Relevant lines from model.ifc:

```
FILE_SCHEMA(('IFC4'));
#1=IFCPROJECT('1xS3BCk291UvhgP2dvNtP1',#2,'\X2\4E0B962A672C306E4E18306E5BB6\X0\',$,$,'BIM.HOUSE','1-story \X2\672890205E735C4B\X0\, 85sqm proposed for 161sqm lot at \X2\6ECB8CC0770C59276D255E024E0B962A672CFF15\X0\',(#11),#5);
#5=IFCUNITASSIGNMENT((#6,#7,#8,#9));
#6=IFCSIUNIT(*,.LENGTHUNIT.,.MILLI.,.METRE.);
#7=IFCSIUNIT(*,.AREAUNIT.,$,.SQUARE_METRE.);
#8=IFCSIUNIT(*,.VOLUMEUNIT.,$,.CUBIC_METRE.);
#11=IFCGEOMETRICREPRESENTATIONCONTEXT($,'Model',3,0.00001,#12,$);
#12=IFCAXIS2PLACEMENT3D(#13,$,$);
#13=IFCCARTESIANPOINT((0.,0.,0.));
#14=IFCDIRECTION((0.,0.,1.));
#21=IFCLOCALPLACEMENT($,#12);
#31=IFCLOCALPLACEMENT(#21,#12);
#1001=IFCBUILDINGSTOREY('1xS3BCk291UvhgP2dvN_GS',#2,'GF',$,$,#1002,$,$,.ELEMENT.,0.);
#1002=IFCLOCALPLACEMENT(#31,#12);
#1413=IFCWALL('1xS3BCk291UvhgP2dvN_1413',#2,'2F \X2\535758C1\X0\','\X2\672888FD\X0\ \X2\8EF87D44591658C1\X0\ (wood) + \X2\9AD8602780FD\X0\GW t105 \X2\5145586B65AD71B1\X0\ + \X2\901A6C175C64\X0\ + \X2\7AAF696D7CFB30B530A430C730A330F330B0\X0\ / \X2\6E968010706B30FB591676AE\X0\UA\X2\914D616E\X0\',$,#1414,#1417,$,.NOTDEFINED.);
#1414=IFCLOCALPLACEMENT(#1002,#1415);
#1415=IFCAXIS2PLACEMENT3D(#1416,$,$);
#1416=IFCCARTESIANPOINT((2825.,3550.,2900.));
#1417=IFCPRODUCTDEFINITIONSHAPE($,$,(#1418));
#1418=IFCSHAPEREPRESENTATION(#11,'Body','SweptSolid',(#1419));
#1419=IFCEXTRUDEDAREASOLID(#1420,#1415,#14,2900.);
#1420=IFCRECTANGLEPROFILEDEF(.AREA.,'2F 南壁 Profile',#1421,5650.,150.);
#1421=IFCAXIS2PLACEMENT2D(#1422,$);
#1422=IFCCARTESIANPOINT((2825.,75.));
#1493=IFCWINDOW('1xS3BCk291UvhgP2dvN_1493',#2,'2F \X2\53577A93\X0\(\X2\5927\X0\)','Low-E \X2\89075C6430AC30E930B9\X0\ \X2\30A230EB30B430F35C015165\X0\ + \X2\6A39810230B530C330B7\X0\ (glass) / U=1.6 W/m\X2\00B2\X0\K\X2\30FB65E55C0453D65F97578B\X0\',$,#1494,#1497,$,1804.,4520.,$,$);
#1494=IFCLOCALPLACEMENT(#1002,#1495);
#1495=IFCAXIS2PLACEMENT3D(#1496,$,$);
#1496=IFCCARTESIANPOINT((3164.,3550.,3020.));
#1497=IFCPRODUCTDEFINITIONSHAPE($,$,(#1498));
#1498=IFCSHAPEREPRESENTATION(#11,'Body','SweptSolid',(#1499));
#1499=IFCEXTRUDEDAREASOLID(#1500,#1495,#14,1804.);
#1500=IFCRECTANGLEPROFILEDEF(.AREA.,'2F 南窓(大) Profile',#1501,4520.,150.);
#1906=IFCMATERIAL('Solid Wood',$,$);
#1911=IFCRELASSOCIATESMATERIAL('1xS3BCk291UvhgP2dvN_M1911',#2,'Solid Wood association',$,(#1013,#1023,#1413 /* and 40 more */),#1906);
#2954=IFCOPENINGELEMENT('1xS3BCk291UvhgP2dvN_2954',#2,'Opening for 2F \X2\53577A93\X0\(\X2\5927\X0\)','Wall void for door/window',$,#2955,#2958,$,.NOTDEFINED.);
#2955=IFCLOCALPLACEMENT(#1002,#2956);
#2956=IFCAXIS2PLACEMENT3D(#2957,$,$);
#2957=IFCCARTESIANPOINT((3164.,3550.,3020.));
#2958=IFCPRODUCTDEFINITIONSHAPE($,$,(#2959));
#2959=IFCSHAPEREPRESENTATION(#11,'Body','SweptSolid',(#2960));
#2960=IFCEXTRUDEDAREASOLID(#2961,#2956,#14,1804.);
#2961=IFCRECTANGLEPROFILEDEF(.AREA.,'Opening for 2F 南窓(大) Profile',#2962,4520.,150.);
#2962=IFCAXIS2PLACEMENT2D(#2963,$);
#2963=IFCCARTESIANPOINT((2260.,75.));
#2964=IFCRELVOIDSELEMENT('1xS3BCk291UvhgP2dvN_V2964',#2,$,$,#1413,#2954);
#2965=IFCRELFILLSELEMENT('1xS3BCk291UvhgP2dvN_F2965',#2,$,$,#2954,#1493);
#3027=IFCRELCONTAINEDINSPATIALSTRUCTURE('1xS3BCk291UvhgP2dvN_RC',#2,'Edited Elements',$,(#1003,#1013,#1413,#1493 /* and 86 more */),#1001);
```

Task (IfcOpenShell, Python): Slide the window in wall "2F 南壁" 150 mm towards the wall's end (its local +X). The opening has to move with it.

```python
import ifcopenshell
import ifcopenshell.api.geometry
import ifcopenshell.util.placement

model = ifcopenshell.open("model.ifc")

window = model.by_id(1493)
opening = window.FillsVoids[0].RelatingOpeningElement
wall = opening.VoidsElements[0].RelatingBuildingElement

wall_matrix = ifcopenshell.util.placement.get_local_placement(wall.ObjectPlacement)
shift = wall_matrix[:3, 0] * 150.0
before = ifcopenshell.util.placement.get_local_placement(window.ObjectPlacement)[:3, 3].copy()

# The window is not placed relative to its opening, so move both.
for product in (opening, window):
    matrix = ifcopenshell.util.placement.get_local_placement(product.ObjectPlacement)
    matrix[:3, 3] += shift
    ifcopenshell.api.geometry.edit_object_placement(model, product=product, matrix=matrix, is_si=False)

after = ifcopenshell.util.placement.get_local_placement(window.ObjectPlacement)[:3, 3]
print("window moved by", (after - before).round(3) + 0.0)

model.write("model_v2.ifc")
```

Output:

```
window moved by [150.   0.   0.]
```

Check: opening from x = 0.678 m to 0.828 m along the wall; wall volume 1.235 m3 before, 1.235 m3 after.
